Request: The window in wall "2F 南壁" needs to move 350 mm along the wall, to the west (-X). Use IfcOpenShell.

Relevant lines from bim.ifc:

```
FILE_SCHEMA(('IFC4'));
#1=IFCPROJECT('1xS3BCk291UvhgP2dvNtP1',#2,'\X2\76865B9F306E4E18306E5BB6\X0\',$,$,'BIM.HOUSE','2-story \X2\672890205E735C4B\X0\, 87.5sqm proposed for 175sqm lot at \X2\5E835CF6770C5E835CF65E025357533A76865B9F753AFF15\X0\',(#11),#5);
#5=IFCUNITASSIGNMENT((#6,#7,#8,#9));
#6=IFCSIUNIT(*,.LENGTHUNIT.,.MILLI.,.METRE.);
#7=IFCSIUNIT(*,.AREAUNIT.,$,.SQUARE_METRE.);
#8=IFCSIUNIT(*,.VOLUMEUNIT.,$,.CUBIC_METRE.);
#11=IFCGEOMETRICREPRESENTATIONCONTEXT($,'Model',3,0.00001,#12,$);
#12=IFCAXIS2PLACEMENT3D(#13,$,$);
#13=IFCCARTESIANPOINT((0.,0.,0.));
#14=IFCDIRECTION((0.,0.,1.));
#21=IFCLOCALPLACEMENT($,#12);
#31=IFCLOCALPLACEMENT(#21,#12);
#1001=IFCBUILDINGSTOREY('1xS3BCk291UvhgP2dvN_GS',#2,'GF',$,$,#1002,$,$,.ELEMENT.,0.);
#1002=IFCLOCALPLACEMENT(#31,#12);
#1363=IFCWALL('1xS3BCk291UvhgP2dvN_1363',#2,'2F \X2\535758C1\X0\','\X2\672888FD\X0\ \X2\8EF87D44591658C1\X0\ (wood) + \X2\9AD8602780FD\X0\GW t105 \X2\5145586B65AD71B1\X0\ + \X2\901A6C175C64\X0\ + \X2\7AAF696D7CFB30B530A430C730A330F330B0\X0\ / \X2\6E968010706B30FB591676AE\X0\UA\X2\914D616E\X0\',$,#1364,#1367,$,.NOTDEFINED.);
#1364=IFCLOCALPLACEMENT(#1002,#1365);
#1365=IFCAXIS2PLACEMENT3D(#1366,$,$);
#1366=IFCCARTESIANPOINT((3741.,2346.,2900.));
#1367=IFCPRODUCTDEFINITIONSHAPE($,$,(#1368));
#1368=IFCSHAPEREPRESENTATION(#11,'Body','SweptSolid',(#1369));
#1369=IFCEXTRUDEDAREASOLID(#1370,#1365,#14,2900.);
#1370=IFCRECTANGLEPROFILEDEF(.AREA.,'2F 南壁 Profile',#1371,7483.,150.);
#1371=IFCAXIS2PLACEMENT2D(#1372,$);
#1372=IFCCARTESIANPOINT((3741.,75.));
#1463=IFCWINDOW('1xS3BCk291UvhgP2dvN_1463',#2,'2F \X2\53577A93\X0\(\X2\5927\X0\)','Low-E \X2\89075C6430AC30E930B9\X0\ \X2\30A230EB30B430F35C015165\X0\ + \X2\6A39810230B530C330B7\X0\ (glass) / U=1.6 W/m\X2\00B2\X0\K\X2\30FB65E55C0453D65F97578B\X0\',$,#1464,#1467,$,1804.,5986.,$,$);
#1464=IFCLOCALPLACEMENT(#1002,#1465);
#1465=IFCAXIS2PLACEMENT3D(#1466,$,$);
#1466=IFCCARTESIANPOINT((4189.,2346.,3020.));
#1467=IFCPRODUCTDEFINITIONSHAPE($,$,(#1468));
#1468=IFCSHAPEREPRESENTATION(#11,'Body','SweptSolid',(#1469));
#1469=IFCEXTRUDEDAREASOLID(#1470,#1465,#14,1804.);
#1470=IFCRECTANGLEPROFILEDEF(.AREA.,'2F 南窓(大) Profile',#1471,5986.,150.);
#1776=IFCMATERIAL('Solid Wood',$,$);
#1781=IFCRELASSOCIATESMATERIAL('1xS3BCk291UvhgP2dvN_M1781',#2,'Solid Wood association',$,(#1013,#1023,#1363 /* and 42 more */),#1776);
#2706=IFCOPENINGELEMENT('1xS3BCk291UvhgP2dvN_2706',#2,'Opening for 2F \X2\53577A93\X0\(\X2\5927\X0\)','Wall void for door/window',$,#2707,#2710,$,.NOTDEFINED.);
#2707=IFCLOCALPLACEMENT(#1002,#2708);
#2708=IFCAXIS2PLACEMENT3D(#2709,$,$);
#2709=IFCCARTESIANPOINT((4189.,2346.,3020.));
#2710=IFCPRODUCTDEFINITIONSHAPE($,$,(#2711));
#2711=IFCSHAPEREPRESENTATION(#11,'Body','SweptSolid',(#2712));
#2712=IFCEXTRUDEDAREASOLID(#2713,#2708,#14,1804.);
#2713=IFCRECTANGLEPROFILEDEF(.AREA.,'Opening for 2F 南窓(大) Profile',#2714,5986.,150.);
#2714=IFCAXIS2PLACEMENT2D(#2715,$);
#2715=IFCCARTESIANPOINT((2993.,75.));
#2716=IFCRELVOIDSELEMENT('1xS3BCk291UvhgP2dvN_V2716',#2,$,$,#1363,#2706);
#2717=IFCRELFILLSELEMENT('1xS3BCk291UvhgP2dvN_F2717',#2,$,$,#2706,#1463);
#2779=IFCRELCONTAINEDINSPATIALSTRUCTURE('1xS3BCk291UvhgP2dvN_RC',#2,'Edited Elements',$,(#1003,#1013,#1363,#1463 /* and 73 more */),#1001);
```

```python
import ifcopenshell
import ifcopenshell.api.geometry
import ifcopenshell.util.placement

model = ifcopenshell.open("bim.ifc")

window = model.by_guid("1xS3BCk291UvhgP2dvN_1463")
opening = window.FillsVoids[0].RelatingOpeningElement
wall = opening.VoidsElements[0].RelatingBuildingElement

wall_matrix = ifcopenshell.util.placement.get_local_placement(wall.ObjectPlacement)
shift = wall_matrix[:3, 0] * -350.0
before = ifcopenshell.util.placement.get_local_placement(window.ObjectPlacement)[:3, 3].copy()

# The window is not placed relative to its opening, so move both.
for product in (opening, window):
    matrix = ifcopenshell.util.placement.get_local_placement(product.ObjectPlacement)
    matrix[:3, 3] += shift
    ifcopenshell.api.geometry.edit_object_placement(model, product=product, matrix=matrix, is_si=False)

after = ifcopenshell.util.placement.get_local_placement(window.ObjectPlacement)[:3, 3]
print("window moved by", (after - before).round(3) + 0.0)

model.write("bim_edited.ifc")
```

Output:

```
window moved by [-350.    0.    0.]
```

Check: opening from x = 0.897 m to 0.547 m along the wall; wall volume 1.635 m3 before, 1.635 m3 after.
